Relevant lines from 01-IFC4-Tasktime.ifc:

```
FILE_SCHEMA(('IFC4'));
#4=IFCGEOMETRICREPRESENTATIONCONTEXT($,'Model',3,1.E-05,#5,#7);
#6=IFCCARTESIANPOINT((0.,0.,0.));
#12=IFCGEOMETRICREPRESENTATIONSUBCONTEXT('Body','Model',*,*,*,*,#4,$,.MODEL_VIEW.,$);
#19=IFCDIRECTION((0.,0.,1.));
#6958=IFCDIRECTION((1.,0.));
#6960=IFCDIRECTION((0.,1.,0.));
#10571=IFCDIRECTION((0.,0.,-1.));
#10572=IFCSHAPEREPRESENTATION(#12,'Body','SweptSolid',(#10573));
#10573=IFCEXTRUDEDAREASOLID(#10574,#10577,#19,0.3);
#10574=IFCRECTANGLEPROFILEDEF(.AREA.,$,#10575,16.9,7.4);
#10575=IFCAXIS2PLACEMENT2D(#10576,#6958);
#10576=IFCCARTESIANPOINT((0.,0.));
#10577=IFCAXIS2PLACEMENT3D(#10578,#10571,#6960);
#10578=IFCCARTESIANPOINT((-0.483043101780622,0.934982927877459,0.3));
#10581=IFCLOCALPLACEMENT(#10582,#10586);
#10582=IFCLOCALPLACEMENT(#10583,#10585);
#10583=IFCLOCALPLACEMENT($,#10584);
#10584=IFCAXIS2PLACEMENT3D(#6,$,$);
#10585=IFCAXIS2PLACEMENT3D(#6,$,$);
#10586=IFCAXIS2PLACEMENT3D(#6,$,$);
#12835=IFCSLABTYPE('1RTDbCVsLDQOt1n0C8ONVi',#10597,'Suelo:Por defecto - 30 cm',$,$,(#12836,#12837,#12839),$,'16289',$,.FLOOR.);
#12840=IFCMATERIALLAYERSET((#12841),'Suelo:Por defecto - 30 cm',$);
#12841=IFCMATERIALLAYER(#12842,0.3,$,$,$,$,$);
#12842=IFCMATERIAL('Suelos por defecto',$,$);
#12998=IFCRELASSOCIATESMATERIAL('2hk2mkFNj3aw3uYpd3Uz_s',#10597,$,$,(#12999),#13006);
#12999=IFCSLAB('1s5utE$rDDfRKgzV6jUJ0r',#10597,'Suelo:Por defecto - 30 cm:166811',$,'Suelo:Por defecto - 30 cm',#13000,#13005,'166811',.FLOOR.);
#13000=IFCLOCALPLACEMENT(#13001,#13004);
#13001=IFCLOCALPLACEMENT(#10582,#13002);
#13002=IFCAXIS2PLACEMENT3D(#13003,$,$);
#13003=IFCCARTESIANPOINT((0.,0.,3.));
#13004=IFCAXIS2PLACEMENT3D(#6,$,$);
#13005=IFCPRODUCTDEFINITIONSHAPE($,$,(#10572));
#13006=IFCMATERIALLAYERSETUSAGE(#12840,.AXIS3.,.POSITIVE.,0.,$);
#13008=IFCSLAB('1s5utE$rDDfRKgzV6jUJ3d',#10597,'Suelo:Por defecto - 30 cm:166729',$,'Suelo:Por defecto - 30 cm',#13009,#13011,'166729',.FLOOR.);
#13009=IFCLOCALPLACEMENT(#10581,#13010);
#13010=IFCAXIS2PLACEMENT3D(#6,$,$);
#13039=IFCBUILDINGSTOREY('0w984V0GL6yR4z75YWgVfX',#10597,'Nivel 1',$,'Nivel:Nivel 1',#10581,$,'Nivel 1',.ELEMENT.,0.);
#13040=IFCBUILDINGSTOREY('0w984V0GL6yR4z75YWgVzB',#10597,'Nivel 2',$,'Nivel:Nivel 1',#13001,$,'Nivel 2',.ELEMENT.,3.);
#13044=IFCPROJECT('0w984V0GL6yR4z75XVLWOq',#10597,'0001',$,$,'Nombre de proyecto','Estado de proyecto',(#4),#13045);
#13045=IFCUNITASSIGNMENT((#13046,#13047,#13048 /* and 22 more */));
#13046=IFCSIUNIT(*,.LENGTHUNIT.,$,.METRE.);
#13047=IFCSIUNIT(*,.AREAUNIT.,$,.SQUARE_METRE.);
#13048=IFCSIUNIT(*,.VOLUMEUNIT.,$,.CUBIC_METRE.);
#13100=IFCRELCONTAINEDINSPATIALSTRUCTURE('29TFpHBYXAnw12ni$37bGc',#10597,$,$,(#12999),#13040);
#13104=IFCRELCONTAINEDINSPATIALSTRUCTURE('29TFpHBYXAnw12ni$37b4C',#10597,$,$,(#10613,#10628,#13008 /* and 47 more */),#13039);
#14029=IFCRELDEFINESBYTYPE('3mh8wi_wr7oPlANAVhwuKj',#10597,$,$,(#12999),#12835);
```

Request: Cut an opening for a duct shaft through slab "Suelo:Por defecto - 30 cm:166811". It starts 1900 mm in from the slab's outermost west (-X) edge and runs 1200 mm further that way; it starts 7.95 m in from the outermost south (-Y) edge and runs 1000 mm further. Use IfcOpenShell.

```python
import numpy as np
import ifcopenshell
import ifcopenshell.api.feature
import ifcopenshell.api.geometry
import ifcopenshell.api.root
import ifcopenshell.geom
import ifcopenshell.util.placement
import ifcopenshell.util.representation
import ifcopenshell.util.shape
import ifcopenshell.util.unit

model = ifcopenshell.open("01-IFC4-Tasktime.ifc")
unit_scale = ifcopenshell.util.unit.calculate_unit_scale(model)
settings = ifcopenshell.geom.settings()


def volume(element):
    """Net volume in cubic metres, openings subtracted."""
    shape = ifcopenshell.geom.create_shape(settings, element)
    return ifcopenshell.util.shape.get_volume(shape.geometry)


slab = model.by_guid("1s5utE$rDDfRKgzV6jUJ0r")
before = volume(slab)

# Extent in the slab's own axes, in metres. The edges named are its -X and -Y sides.
slab_shape = ifcopenshell.geom.create_shape(settings, slab)
vertices = ifcopenshell.util.shape.get_vertices(slab_shape.geometry)
x_min, y_min, bottom = vertices.min(axis=0)
top = vertices[:, 2].max()

opening = ifcopenshell.api.root.create_entity(model, ifc_class="IfcOpeningElement", name="Duct shaft opening", predefined_type="OPENING")
context = ifcopenshell.util.representation.get_context(model, "Model", "Body", "MODEL_VIEW")
width, depth = 1.2, 1
outline = [(0.0, 0.0), (width, 0.0), (width, depth), (0.0, depth), (0.0, 0.0)]
# Overshoot both faces by 50 mm so the cut is clean.
shape = ifcopenshell.api.geometry.add_slab_representation(
    model, context=context, depth=top - bottom + 0.1, polyline=outline
)
ifcopenshell.api.geometry.assign_representation(model, product=opening, representation=shape)

matrix = ifcopenshell.util.placement.get_local_placement(slab.ObjectPlacement)
matrix[:, 3] = matrix @ np.append(np.array([x_min + 1.9, y_min + 7.95, bottom - 0.05]) / unit_scale, 1.0)
ifcopenshell.api.geometry.edit_object_placement(model, product=opening, matrix=matrix, is_si=False)
ifcopenshell.api.feature.add_feature(model, feature=opening, element=slab)

after = volume(slab)

print(f"slab volume {before:.3f} -> {after:.3f} m3")

model.write("01-IFC4-Tasktime-out.ifc")
```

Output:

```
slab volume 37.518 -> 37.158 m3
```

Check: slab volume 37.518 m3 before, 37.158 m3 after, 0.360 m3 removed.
